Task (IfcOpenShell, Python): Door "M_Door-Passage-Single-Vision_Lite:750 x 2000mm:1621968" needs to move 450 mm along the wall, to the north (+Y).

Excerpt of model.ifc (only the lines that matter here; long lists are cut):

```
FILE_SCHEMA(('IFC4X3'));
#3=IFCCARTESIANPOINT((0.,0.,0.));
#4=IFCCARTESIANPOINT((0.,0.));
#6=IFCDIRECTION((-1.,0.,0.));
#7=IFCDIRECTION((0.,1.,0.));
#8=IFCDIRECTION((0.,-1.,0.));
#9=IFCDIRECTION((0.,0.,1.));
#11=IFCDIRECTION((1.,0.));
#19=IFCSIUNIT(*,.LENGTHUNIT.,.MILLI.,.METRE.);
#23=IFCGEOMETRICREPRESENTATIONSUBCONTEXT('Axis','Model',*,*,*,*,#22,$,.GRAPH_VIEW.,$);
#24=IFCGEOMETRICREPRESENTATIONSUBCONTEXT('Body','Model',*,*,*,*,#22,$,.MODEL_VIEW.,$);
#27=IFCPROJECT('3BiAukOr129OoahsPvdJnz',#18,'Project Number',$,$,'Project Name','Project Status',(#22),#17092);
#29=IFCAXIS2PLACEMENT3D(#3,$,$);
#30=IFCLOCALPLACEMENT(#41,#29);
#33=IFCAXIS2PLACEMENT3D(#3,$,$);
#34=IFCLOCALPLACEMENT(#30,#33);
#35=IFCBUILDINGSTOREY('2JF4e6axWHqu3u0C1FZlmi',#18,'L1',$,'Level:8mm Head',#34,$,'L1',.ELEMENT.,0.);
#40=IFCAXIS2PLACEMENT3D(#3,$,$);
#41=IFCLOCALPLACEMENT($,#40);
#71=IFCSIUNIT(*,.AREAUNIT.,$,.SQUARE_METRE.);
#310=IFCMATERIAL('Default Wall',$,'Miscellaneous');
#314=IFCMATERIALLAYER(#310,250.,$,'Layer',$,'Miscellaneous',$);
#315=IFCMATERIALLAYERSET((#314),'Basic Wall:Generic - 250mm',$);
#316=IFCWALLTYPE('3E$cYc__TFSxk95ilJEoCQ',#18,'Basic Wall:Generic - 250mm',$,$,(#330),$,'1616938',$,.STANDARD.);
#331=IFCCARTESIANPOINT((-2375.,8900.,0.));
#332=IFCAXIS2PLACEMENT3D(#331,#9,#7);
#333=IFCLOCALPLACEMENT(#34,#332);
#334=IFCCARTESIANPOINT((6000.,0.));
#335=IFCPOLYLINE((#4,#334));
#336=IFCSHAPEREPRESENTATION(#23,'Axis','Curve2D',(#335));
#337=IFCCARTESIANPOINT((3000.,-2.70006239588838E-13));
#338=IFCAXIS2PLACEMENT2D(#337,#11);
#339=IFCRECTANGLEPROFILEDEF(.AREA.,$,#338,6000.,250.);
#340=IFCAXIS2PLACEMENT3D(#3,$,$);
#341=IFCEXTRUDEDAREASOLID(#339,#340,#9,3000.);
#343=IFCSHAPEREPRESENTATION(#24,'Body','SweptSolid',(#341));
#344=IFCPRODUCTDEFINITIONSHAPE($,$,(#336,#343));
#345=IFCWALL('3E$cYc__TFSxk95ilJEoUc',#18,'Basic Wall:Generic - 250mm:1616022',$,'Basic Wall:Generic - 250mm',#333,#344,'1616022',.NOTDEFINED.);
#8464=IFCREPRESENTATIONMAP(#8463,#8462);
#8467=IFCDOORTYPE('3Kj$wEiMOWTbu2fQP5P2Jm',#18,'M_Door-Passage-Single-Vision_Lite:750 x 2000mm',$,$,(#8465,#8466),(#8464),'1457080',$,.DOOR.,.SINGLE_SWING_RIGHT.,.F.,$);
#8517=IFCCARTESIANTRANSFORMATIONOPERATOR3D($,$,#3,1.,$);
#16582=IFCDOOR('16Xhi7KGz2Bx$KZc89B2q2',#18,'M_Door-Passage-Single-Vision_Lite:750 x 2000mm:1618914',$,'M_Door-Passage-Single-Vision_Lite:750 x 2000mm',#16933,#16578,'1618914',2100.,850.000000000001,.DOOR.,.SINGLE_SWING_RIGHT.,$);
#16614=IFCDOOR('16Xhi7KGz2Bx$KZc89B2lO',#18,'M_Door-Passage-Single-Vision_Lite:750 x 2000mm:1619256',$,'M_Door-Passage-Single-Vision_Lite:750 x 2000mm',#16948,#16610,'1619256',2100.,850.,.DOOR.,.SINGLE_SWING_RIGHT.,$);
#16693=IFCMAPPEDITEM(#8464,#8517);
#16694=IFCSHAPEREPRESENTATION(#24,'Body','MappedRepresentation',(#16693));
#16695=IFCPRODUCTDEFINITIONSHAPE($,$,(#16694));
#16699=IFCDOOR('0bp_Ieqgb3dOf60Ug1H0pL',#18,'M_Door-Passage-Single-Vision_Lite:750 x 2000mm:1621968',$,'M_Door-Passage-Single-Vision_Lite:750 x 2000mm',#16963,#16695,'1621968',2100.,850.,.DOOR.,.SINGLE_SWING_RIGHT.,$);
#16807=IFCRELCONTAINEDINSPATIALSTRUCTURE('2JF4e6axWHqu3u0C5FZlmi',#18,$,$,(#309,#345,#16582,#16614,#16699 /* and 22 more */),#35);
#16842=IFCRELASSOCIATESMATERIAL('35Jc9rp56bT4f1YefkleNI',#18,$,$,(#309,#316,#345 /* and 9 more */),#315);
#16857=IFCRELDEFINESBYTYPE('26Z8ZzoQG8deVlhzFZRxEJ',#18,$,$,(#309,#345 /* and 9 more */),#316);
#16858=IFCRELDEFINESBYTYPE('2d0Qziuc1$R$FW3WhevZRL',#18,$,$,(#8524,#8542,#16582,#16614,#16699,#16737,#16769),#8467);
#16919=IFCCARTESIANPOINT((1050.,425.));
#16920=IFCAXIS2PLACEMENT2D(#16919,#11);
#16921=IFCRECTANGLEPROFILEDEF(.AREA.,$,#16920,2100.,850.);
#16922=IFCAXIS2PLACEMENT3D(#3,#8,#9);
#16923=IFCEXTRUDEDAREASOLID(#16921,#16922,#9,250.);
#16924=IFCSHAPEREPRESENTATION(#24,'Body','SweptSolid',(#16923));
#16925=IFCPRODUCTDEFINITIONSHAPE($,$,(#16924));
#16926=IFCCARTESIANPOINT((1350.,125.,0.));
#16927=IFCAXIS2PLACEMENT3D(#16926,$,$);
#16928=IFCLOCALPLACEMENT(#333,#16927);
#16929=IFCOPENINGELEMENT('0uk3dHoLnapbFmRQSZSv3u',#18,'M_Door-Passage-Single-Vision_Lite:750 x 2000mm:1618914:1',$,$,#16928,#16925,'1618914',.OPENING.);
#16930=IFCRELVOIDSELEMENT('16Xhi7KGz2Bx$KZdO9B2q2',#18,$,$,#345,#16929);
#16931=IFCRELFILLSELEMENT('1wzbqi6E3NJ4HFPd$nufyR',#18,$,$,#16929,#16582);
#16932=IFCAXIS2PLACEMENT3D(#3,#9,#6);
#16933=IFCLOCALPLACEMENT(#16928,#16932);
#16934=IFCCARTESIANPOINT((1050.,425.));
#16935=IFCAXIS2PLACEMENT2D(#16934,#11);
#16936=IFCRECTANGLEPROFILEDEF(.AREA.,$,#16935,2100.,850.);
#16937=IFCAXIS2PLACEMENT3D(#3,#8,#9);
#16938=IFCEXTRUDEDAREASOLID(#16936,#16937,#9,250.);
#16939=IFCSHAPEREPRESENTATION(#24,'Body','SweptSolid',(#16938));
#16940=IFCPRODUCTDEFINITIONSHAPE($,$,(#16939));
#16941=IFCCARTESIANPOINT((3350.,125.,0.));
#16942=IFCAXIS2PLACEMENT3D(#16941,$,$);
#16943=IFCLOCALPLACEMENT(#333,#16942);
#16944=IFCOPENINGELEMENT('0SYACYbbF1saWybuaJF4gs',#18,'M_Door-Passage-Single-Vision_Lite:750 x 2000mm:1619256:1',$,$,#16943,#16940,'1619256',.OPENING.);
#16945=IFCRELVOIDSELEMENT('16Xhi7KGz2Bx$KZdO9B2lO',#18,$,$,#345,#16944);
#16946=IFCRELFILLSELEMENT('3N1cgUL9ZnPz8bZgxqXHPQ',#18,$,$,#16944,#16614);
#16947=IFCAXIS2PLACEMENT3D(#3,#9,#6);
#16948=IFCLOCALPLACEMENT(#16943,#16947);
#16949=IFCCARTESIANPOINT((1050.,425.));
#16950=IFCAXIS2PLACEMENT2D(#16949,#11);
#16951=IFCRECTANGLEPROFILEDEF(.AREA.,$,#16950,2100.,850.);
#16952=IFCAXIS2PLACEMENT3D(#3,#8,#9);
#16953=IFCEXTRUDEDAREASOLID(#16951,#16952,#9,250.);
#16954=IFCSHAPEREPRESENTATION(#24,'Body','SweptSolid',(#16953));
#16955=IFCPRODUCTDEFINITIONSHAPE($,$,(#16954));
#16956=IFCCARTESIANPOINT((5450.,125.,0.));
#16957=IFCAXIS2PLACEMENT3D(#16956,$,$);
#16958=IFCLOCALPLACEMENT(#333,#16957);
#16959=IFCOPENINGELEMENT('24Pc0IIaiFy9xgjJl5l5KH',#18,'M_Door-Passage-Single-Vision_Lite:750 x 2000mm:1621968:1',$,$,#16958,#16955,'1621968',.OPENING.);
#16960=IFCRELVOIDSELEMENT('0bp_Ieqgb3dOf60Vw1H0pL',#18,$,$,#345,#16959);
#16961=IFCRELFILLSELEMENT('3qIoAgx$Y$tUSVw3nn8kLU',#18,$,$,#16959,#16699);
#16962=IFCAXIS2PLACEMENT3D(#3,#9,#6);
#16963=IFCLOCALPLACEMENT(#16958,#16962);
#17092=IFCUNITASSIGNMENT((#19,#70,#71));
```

```python
import ifcopenshell
import ifcopenshell.api.geometry
import ifcopenshell.util.placement
import ifcopenshell.util.unit

model = ifcopenshell.open("model.ifc")
unit_scale = ifcopenshell.util.unit.calculate_unit_scale(model)

door = model.by_guid("0bp_Ieqgb3dOf60Ug1H0pL")
opening = door.FillsVoids[0].RelatingOpeningElement
wall = opening.VoidsElements[0].RelatingBuildingElement

wall_matrix = ifcopenshell.util.placement.get_local_placement(wall.ObjectPlacement)
shift = wall_matrix[:3, 0] * 0.45 / unit_scale
before = ifcopenshell.util.placement.get_local_placement(door.ObjectPlacement)[:3, 3].copy()

# The door is placed relative to its opening, so it follows when the opening moves.
matrix = ifcopenshell.util.placement.get_local_placement(opening.ObjectPlacement)
matrix[:3, 3] += shift
ifcopenshell.api.geometry.edit_object_placement(
    model, product=opening, matrix=matrix, is_si=False, should_transform_children=True
)

after = ifcopenshell.util.placement.get_local_placement(door.ObjectPlacement)[:3, 3]
print("door moved by", (after - before).round(3) + 0.0)

model.write("model_updated.ifc")
```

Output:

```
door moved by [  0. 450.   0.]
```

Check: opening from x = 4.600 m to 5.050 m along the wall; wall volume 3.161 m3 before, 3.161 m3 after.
